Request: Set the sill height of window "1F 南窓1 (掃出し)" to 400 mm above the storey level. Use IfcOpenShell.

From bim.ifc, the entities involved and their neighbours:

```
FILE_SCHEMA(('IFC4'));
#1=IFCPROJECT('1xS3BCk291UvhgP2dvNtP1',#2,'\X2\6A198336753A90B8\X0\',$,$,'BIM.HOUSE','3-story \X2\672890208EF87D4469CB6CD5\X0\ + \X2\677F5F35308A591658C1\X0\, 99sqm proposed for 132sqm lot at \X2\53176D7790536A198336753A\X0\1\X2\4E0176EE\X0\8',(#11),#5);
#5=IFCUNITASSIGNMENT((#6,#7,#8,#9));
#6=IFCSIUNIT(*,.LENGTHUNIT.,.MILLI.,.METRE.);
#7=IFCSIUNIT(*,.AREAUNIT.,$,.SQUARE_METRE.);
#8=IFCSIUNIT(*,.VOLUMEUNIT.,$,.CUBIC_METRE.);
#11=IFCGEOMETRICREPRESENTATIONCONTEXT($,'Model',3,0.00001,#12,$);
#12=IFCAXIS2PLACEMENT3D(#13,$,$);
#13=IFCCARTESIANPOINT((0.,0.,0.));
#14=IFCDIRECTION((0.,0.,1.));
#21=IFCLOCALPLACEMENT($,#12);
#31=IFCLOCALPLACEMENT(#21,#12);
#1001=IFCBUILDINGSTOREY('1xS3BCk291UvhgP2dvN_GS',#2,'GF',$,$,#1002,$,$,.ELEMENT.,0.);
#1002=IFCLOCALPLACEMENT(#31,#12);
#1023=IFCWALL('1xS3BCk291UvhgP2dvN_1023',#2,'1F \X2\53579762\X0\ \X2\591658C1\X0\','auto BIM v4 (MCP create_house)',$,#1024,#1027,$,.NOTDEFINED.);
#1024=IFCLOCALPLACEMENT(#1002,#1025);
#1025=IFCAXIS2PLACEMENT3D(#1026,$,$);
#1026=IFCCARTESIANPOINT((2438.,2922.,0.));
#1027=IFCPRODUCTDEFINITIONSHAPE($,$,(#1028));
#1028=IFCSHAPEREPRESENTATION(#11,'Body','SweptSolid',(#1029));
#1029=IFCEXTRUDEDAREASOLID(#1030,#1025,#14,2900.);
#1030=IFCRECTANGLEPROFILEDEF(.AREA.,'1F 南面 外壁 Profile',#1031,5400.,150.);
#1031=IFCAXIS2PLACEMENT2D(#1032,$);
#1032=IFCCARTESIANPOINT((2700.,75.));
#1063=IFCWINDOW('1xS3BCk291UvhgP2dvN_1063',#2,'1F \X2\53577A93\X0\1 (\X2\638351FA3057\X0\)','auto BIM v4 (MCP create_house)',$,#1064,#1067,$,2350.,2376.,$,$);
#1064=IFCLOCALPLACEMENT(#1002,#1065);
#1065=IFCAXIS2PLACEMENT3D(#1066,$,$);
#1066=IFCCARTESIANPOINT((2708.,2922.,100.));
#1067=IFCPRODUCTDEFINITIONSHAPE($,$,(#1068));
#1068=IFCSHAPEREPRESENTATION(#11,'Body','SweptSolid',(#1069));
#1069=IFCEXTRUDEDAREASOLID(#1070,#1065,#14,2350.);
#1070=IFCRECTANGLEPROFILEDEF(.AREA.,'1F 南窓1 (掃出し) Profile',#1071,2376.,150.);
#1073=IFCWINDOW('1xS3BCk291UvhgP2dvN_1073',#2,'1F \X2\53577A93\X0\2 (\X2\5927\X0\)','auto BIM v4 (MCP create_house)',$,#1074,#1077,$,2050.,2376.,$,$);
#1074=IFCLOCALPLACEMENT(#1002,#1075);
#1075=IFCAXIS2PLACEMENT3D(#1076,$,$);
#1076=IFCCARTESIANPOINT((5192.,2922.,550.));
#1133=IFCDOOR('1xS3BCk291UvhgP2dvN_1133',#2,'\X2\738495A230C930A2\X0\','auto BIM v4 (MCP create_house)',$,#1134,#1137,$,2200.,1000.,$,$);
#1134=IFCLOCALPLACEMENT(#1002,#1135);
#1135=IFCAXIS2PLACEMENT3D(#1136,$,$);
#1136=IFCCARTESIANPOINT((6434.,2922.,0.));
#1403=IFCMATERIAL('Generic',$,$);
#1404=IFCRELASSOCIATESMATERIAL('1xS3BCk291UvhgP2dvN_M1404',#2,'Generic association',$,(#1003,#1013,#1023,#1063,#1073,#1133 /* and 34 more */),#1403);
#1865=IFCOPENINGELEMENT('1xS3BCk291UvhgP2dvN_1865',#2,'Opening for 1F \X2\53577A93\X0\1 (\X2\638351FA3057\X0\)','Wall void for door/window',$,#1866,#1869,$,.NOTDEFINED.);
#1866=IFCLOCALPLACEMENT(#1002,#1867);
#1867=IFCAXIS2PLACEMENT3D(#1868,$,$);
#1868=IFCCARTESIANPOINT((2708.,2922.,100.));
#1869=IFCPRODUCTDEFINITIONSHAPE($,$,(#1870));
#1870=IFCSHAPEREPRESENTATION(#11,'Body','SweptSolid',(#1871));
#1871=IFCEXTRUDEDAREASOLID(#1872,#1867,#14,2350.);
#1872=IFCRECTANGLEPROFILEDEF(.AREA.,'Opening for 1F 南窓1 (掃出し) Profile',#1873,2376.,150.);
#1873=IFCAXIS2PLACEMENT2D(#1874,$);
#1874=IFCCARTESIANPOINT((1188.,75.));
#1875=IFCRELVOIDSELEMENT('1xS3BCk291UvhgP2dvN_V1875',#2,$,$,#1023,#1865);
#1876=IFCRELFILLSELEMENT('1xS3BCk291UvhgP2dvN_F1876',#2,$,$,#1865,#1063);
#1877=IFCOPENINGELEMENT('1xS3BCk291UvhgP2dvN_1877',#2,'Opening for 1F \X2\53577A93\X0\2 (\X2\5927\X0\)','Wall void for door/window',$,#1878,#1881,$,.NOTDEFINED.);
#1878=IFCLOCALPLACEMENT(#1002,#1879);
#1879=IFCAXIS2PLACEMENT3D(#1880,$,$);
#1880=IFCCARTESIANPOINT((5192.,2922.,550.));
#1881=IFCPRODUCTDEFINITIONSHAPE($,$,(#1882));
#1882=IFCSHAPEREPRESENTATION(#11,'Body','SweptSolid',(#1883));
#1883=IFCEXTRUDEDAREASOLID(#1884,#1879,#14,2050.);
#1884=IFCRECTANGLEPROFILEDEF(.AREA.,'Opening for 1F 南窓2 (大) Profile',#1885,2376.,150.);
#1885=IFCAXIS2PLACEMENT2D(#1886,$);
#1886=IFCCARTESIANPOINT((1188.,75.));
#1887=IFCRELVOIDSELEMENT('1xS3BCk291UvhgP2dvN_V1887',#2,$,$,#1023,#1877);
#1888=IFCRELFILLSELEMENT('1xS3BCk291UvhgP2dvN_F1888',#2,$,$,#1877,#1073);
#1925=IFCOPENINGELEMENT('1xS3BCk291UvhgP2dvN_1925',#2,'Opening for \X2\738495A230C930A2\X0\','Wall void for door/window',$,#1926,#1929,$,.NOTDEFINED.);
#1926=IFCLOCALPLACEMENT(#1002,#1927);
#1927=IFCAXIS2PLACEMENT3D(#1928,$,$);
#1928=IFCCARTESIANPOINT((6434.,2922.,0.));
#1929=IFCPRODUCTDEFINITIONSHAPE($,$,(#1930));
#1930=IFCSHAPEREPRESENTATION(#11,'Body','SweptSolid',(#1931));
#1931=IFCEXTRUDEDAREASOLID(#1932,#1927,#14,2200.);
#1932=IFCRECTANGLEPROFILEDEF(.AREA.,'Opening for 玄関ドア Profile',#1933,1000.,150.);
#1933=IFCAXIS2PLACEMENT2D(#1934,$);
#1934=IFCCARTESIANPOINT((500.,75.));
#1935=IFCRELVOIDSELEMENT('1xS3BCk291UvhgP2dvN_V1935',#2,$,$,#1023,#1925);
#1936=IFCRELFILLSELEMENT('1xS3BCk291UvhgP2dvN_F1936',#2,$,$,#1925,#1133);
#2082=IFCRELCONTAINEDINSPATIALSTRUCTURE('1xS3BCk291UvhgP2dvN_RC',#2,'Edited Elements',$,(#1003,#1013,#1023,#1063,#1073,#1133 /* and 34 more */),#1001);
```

```python
import numpy as np
import ifcopenshell
import ifcopenshell.api.geometry
import ifcopenshell.geom
import ifcopenshell.util.element
import ifcopenshell.util.placement
import ifcopenshell.util.shape
import ifcopenshell.util.unit

model = ifcopenshell.open("bim.ifc")
unit_scale = ifcopenshell.util.unit.calculate_unit_scale(model)

window = model.by_guid("1xS3BCk291UvhgP2dvN_1063")
opening = window.FillsVoids[0].RelatingOpeningElement
storey = ifcopenshell.util.element.get_container(window, ifc_class="IfcBuildingStorey")
level = ifcopenshell.util.placement.get_local_placement(storey.ObjectPlacement)[2, 3]

# The opening's origin need not be at the sill, so measure its lowest point.
shape = ifcopenshell.geom.create_shape(ifcopenshell.geom.settings(), opening)
bottom = ifcopenshell.util.shape.get_shape_bottom_elevation(shape, shape.geometry) / unit_scale
dz = level + 0.4 / unit_scale - bottom

shift = np.array([0.0, 0.0, dz])
# The window is not placed relative to its opening, so move both.
for product in (opening, window):
    matrix = ifcopenshell.util.placement.get_local_placement(product.ObjectPlacement)
    matrix[:3, 3] += shift
    ifcopenshell.api.geometry.edit_object_placement(model, product=product, matrix=matrix, is_si=False)

print(f"moved by {dz * unit_scale:+.3f} m")

model.write("bim-out.ifc")
```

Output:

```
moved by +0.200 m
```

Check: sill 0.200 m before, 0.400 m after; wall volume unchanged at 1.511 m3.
